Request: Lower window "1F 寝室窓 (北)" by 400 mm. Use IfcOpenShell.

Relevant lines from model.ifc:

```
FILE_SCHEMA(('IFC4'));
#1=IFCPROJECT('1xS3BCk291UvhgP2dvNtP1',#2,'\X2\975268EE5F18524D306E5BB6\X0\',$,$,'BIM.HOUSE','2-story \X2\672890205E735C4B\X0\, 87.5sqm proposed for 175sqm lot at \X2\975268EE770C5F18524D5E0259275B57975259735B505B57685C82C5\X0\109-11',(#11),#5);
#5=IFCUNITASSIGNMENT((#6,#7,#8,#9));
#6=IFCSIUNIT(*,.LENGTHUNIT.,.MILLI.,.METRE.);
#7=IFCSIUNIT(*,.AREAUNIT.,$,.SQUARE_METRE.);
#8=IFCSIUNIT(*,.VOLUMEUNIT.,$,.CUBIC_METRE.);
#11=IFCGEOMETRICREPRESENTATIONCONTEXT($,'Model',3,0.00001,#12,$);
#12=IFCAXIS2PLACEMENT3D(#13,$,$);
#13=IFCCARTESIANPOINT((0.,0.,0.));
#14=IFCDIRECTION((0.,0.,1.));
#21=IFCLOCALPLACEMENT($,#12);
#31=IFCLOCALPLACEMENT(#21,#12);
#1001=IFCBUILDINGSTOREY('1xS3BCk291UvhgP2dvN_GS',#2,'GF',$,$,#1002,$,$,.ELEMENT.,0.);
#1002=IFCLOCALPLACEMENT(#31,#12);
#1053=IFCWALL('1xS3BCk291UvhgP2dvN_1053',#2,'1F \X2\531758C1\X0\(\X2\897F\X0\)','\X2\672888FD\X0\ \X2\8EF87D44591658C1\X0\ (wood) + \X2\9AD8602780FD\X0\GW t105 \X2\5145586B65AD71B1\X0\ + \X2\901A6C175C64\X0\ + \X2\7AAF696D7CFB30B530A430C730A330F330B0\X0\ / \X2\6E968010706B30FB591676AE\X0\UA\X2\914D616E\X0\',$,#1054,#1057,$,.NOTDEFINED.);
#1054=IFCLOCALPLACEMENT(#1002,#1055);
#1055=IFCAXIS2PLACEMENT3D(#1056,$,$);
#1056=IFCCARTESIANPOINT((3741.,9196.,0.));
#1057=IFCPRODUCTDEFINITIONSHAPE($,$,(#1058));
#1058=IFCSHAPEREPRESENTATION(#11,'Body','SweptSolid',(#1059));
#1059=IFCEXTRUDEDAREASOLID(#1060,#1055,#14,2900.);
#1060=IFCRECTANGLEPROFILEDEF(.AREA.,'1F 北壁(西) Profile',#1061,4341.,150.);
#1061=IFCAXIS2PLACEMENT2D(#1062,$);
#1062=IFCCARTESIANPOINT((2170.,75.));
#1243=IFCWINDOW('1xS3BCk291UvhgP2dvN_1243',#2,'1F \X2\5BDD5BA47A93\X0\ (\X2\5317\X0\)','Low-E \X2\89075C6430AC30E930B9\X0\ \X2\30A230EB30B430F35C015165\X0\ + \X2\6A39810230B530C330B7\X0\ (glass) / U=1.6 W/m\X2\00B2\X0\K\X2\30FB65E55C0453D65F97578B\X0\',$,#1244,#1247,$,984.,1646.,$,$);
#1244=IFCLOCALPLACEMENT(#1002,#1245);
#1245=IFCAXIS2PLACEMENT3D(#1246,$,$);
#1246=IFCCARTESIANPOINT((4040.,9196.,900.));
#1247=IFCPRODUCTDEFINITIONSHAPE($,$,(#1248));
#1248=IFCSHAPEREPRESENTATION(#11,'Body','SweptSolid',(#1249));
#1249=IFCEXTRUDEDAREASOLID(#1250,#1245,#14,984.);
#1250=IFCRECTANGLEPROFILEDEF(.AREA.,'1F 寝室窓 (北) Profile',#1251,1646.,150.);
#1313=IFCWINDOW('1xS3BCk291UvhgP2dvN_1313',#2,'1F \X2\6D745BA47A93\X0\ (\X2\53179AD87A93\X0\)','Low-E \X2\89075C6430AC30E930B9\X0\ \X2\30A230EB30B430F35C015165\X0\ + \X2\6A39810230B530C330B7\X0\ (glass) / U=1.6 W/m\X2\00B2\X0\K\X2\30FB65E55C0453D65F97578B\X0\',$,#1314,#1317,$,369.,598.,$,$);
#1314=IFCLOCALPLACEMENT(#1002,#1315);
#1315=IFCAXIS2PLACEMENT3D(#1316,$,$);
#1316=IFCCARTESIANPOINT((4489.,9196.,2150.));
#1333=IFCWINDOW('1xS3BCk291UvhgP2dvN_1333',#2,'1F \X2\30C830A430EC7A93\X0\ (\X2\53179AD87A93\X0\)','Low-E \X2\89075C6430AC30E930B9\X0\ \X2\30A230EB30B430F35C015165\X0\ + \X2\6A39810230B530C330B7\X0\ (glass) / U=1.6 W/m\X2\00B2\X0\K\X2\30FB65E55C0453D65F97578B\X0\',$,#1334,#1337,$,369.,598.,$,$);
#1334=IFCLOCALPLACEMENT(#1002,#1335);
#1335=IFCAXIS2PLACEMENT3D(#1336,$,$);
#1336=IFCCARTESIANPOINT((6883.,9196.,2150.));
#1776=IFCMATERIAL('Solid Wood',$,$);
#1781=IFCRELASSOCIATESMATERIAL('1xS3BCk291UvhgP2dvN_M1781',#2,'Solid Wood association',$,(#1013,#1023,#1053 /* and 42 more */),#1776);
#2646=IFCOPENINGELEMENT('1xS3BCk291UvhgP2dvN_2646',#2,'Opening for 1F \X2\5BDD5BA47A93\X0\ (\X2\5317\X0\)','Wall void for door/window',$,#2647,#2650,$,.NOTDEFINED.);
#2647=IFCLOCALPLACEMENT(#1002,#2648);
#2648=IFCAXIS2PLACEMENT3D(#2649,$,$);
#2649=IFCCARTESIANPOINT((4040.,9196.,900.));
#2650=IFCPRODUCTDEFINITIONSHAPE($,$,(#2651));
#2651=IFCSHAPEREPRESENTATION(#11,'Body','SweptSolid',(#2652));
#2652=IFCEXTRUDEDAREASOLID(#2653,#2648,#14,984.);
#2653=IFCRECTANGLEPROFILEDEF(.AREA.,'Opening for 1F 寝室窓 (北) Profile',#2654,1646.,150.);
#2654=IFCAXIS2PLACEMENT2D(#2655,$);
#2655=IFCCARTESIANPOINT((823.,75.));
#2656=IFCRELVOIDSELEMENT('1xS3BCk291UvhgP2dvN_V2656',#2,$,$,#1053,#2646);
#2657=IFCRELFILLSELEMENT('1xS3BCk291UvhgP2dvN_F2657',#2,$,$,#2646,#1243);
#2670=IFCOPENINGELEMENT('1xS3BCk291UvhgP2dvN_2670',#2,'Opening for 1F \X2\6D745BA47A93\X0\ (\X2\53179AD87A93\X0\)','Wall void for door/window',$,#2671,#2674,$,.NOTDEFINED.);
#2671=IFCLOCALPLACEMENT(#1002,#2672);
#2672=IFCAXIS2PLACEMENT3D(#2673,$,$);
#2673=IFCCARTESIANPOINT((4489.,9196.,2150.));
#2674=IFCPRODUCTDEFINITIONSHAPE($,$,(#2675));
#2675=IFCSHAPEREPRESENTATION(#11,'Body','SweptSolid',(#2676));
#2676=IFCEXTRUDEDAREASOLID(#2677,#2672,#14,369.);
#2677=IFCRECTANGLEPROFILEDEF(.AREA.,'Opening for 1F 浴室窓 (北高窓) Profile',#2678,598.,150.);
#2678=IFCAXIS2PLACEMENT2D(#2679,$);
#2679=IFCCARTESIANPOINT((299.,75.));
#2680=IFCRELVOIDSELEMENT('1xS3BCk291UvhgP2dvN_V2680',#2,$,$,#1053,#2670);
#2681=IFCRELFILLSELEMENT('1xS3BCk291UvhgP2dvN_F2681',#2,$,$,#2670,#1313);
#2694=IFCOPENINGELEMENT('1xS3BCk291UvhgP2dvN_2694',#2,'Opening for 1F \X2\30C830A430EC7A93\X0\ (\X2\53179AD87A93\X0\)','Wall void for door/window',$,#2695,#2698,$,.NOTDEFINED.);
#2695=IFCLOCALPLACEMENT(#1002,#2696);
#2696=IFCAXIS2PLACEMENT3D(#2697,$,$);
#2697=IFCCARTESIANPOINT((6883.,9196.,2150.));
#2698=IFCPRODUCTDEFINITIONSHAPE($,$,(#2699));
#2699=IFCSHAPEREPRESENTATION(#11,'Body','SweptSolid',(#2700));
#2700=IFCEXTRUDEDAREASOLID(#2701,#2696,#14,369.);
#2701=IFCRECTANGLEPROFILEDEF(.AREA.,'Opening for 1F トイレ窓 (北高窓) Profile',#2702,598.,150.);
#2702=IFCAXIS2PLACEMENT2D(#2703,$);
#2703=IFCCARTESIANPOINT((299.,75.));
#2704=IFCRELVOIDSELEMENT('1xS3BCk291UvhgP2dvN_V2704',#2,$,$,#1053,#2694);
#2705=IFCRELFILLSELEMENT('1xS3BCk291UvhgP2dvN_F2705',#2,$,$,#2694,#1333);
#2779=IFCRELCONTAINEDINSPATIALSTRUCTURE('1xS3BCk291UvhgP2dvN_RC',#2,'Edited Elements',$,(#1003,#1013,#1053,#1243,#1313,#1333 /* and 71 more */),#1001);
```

```python
import numpy as np
import ifcopenshell
import ifcopenshell.api.geometry
import ifcopenshell.util.placement
import ifcopenshell.util.unit

model = ifcopenshell.open("model.ifc")
unit_scale = ifcopenshell.util.unit.calculate_unit_scale(model)

window = model.by_guid("1xS3BCk291UvhgP2dvN_1243")
opening = window.FillsVoids[0].RelatingOpeningElement
dz = -400.0

shift = np.array([0.0, 0.0, dz])
# The window is not placed relative to its opening, so move both.
for product in (opening, window):
    matrix = ifcopenshell.util.placement.get_local_placement(product.ObjectPlacement)
    matrix[:3, 3] += shift
    ifcopenshell.api.geometry.edit_object_placement(model, product=product, matrix=matrix, is_si=False)

print(f"moved by {dz * unit_scale:+.3f} m")

model.write("model_rev.ifc")
```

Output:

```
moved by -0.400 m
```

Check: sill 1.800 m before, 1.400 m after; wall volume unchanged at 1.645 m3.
